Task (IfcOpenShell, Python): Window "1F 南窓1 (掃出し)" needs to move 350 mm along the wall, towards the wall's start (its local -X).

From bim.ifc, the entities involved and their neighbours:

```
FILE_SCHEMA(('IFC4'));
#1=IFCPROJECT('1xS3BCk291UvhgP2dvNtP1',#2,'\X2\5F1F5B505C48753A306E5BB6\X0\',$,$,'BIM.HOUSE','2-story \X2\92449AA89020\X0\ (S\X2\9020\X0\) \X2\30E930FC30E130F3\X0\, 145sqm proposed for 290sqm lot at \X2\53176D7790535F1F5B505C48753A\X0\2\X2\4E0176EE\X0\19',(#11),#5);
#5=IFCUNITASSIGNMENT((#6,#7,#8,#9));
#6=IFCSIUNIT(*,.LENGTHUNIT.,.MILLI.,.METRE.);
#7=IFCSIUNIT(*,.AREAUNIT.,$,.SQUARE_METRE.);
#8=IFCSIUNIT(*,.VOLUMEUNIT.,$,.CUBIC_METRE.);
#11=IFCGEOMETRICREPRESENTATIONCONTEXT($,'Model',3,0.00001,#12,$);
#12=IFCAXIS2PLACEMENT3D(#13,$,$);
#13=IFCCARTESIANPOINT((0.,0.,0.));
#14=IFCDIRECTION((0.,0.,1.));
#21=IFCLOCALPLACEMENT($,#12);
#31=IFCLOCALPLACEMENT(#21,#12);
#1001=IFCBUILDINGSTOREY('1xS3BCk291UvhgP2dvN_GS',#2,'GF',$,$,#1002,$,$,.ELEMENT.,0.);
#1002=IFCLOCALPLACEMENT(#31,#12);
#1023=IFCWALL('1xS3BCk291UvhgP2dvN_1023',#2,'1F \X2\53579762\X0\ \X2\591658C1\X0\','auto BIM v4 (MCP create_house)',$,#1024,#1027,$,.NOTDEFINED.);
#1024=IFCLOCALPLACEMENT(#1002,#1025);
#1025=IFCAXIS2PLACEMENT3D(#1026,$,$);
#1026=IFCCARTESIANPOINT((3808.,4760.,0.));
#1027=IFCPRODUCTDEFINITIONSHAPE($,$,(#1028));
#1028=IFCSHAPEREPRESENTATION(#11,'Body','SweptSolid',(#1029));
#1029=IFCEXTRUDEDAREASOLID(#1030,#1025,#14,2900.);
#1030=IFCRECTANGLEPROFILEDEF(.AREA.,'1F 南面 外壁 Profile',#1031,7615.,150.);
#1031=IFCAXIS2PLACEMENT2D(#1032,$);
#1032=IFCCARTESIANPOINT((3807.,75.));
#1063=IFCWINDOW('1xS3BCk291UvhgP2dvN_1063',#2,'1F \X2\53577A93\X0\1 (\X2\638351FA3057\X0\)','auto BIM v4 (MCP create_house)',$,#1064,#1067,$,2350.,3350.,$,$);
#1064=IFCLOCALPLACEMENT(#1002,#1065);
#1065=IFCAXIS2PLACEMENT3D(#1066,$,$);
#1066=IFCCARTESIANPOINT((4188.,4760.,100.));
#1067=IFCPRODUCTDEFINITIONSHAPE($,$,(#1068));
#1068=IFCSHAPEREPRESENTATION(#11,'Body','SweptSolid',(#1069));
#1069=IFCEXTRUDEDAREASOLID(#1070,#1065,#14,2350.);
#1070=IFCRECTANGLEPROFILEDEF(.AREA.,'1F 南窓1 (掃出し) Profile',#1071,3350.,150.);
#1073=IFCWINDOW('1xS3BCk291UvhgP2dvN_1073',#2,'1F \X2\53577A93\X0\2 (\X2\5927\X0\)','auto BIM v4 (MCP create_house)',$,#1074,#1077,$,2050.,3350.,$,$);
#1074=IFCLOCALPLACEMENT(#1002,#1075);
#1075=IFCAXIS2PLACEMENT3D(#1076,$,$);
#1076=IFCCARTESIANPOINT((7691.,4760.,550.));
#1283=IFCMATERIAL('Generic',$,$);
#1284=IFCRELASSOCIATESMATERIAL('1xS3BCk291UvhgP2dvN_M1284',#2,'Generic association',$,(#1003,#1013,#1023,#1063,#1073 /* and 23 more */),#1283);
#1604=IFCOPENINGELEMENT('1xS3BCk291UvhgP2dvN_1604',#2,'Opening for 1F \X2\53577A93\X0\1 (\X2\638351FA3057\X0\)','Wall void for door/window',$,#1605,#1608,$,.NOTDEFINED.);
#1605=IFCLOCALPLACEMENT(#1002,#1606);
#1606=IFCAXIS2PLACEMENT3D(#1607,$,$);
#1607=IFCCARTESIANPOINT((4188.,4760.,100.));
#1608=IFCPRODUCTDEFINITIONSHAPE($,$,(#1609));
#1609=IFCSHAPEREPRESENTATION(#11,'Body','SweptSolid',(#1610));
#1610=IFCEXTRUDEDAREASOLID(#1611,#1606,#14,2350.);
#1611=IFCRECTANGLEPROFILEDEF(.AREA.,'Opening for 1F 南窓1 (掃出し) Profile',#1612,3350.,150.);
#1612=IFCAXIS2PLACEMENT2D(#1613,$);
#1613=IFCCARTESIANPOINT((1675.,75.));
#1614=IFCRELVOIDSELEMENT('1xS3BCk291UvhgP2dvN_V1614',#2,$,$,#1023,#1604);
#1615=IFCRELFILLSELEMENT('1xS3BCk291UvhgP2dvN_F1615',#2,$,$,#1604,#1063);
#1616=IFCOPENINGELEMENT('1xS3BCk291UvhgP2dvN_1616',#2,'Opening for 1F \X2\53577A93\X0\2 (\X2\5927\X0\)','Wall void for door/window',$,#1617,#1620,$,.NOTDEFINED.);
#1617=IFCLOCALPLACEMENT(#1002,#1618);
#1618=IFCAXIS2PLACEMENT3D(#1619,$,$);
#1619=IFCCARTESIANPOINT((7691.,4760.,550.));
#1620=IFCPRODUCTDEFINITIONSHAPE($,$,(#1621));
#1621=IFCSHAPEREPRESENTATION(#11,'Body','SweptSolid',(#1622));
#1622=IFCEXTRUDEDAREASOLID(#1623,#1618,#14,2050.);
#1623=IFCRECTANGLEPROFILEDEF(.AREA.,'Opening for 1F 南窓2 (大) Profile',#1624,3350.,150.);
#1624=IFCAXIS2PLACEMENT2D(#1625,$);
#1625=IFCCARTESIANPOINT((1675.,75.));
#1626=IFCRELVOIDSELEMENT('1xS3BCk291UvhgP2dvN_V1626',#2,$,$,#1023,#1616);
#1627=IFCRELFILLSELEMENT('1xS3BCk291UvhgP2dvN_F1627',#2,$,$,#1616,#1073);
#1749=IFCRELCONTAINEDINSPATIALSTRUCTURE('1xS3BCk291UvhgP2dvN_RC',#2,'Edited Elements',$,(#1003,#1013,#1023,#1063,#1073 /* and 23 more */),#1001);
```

```python
import ifcopenshell
import ifcopenshell.api.geometry
import ifcopenshell.util.placement
import ifcopenshell.util.unit

model = ifcopenshell.open("bim.ifc")
unit_scale = ifcopenshell.util.unit.calculate_unit_scale(model)

window = model.by_id(1063)
opening = window.FillsVoids[0].RelatingOpeningElement
wall = opening.VoidsElements[0].RelatingBuildingElement

wall_matrix = ifcopenshell.util.placement.get_local_placement(wall.ObjectPlacement)
shift = wall_matrix[:3, 0] * -0.35 / unit_scale
before = ifcopenshell.util.placement.get_local_placement(window.ObjectPlacement)[:3, 3].copy()

# The window is not placed relative to its opening, so move both.
for product in (opening, window):
    matrix = ifcopenshell.util.placement.get_local_placement(product.ObjectPlacement)
    matrix[:3, 3] += shift
    ifcopenshell.api.geometry.edit_object_placement(model, product=product, matrix=matrix, is_si=False)

after = ifcopenshell.util.placement.get_local_placement(window.ObjectPlacement)[:3, 3]
print("window moved by", (after - before).round(3) + 0.0)

model.write("bim_rev.ifc")
```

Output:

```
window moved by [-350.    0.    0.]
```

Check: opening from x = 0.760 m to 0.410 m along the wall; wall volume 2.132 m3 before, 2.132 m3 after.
